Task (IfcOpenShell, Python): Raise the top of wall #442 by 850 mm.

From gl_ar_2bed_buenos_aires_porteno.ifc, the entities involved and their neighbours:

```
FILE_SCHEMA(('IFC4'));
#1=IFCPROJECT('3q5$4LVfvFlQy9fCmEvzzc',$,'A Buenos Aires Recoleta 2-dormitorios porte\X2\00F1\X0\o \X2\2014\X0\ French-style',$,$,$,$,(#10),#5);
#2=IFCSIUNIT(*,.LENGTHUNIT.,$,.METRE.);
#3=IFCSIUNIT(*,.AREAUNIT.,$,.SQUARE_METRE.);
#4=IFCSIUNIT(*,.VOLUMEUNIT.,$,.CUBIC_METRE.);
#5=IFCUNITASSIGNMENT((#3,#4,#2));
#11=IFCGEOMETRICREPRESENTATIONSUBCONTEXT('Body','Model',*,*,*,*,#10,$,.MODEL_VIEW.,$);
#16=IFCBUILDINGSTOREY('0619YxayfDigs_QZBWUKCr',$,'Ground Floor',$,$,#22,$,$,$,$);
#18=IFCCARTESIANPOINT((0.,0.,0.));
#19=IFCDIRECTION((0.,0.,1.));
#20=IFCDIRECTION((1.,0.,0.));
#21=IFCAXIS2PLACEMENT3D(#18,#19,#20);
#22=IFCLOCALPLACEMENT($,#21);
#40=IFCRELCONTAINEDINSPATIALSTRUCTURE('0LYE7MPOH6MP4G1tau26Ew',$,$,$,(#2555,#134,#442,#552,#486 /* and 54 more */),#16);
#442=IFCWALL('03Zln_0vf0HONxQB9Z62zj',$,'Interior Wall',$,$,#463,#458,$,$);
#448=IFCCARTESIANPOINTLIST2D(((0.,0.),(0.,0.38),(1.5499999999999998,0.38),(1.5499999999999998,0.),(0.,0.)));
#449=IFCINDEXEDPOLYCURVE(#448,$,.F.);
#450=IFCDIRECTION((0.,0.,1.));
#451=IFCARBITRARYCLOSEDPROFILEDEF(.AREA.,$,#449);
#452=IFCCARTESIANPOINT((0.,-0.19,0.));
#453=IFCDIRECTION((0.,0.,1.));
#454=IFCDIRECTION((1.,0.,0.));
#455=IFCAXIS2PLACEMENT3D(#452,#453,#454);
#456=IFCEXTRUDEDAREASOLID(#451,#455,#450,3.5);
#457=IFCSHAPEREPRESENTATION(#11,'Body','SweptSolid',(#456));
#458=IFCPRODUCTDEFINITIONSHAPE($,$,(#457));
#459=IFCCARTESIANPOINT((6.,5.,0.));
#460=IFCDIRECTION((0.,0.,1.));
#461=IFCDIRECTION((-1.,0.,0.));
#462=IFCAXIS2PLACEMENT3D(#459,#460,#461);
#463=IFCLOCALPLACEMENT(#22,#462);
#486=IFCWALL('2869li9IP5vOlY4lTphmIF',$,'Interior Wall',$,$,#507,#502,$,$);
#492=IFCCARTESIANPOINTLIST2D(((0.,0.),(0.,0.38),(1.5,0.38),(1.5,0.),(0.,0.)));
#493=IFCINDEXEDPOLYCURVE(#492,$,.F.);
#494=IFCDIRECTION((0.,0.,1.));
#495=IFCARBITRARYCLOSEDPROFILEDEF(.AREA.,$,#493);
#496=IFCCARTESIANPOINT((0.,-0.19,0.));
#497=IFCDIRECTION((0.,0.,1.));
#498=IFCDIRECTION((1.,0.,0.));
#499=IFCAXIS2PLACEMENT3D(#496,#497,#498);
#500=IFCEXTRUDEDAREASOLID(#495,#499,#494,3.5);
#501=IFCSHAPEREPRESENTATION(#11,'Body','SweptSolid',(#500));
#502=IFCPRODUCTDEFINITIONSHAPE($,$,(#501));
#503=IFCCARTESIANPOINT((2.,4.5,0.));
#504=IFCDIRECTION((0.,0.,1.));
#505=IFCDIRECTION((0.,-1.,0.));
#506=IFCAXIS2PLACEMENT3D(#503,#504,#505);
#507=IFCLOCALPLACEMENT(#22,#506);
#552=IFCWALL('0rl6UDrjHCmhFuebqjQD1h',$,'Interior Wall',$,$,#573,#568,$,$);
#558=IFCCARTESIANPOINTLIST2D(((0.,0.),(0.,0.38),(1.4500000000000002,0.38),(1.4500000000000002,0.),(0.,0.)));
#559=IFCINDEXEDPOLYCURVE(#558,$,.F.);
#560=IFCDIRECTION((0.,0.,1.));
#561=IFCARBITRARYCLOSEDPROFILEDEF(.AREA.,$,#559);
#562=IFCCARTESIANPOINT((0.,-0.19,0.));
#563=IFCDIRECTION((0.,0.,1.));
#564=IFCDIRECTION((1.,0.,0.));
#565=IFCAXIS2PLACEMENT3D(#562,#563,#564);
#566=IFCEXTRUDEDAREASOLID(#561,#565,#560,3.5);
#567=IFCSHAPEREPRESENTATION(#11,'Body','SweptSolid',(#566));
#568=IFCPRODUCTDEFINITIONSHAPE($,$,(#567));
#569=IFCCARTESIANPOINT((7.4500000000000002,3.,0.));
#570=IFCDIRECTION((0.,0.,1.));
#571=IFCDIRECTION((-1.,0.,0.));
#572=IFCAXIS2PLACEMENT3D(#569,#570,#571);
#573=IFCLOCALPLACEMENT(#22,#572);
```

```python
import ifcopenshell
import ifcopenshell.geom
import ifcopenshell.util.representation
import ifcopenshell.util.shape

model = ifcopenshell.open("gl_ar_2bed_buenos_aires_porteno.ifc")
settings = ifcopenshell.geom.settings()


def volume(element):
    """Net volume in cubic metres, openings subtracted."""
    shape = ifcopenshell.geom.create_shape(settings, element)
    return ifcopenshell.util.shape.get_volume(shape.geometry)


wall = model.by_id(442)
before = volume(wall)

body = ifcopenshell.util.representation.get_representation(wall, "Model", "Body")
solid = body.Items[0]
old_height = solid.Depth
solid.Depth += 0.85
after = volume(wall)

print(f"height {old_height:g} -> {solid.Depth:g}, volume {before:.3f} -> {after:.3f} m3")

model.write("gl_ar_2bed_buenos_aires_porteno-out.ifc")
```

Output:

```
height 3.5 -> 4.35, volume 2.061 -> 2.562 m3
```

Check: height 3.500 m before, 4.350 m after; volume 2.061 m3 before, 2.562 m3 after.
